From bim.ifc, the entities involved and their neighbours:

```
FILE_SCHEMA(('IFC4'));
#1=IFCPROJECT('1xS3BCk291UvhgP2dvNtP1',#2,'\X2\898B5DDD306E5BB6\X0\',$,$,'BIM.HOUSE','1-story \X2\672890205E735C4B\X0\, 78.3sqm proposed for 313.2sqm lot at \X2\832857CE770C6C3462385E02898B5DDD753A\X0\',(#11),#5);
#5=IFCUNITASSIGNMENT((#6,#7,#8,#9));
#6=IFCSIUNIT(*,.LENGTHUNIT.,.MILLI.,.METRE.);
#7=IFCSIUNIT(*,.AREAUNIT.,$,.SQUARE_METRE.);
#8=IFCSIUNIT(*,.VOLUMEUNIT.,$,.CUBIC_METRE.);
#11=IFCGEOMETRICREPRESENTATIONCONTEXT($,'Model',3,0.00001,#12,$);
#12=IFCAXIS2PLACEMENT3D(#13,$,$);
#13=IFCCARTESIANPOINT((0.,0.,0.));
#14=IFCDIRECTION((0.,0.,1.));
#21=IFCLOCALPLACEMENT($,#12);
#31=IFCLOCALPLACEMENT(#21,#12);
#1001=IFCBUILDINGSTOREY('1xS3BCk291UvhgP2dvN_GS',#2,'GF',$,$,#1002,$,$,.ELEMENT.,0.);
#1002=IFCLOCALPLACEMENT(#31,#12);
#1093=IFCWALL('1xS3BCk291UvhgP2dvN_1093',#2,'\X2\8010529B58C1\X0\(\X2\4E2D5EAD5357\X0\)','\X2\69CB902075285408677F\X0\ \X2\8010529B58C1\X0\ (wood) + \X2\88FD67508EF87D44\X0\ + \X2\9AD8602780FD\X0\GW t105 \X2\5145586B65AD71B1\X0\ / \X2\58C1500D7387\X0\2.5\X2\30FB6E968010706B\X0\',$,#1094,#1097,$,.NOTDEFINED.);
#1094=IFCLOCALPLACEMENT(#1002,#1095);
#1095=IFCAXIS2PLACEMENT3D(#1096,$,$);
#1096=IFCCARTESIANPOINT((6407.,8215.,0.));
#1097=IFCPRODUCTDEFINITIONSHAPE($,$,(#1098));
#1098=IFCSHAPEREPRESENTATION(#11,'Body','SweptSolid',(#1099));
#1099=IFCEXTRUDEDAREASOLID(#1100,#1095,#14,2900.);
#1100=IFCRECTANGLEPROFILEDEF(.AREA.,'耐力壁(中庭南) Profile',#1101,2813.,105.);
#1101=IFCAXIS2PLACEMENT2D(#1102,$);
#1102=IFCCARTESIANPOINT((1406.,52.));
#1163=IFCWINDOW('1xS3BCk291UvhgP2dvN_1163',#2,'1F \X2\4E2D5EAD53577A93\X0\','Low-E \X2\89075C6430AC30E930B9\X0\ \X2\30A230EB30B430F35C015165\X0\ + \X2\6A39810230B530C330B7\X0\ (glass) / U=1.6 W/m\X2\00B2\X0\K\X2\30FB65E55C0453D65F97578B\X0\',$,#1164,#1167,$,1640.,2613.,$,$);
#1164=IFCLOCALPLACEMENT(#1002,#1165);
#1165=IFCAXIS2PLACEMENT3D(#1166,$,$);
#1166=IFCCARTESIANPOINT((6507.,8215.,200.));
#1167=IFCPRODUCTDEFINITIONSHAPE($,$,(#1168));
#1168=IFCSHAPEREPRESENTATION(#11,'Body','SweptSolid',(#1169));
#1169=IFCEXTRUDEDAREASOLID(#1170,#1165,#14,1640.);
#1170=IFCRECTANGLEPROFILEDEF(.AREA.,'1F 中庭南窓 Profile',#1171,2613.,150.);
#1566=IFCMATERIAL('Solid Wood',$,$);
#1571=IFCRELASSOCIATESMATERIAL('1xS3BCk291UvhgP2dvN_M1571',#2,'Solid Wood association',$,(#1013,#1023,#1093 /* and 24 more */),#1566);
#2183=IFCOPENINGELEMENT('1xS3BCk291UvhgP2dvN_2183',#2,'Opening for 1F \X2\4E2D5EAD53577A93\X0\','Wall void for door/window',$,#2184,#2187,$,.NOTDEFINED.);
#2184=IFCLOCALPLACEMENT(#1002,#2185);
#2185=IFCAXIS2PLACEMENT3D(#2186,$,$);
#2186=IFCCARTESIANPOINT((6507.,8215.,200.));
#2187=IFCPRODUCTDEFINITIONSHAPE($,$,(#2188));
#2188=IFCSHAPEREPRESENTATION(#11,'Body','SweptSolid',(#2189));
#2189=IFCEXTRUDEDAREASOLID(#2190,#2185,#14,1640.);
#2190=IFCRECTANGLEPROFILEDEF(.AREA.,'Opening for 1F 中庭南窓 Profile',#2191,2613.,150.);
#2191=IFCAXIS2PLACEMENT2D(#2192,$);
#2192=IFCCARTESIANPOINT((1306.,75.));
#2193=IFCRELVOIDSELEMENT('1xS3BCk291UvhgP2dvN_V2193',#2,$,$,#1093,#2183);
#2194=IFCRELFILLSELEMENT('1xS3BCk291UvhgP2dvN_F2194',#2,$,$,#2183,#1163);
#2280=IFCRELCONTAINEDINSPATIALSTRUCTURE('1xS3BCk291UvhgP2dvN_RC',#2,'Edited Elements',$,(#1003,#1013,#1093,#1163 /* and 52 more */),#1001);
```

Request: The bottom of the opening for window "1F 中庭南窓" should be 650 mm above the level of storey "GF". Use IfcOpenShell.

```python
import numpy as np
import ifcopenshell
import ifcopenshell.api.geometry
import ifcopenshell.geom
import ifcopenshell.util.element
import ifcopenshell.util.placement
import ifcopenshell.util.shape
import ifcopenshell.util.unit

model = ifcopenshell.open("bim.ifc")
unit_scale = ifcopenshell.util.unit.calculate_unit_scale(model)

window = model.by_id(1163)
opening = window.FillsVoids[0].RelatingOpeningElement
storey = ifcopenshell.util.element.get_container(window, ifc_class="IfcBuildingStorey")
level = ifcopenshell.util.placement.get_local_placement(storey.ObjectPlacement)[2, 3]

# The opening's origin need not be at the sill, so measure its lowest point.
shape = ifcopenshell.geom.create_shape(ifcopenshell.geom.settings(), opening)
bottom = ifcopenshell.util.shape.get_shape_bottom_elevation(shape, shape.geometry) / unit_scale
dz = level + 0.65 / unit_scale - bottom

shift = np.array([0.0, 0.0, dz])
# The window is not placed relative to its opening, so move both.
for product in (opening, window):
    matrix = ifcopenshell.util.placement.get_local_placement(product.ObjectPlacement)
    matrix[:3, 3] += shift
    ifcopenshell.api.geometry.edit_object_placement(model, product=product, matrix=matrix, is_si=False)

print(f"moved by {dz * unit_scale:+.3f} m")

model.write("bim_v2.ifc")
```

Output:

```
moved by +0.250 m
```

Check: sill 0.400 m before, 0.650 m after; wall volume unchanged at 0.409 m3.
